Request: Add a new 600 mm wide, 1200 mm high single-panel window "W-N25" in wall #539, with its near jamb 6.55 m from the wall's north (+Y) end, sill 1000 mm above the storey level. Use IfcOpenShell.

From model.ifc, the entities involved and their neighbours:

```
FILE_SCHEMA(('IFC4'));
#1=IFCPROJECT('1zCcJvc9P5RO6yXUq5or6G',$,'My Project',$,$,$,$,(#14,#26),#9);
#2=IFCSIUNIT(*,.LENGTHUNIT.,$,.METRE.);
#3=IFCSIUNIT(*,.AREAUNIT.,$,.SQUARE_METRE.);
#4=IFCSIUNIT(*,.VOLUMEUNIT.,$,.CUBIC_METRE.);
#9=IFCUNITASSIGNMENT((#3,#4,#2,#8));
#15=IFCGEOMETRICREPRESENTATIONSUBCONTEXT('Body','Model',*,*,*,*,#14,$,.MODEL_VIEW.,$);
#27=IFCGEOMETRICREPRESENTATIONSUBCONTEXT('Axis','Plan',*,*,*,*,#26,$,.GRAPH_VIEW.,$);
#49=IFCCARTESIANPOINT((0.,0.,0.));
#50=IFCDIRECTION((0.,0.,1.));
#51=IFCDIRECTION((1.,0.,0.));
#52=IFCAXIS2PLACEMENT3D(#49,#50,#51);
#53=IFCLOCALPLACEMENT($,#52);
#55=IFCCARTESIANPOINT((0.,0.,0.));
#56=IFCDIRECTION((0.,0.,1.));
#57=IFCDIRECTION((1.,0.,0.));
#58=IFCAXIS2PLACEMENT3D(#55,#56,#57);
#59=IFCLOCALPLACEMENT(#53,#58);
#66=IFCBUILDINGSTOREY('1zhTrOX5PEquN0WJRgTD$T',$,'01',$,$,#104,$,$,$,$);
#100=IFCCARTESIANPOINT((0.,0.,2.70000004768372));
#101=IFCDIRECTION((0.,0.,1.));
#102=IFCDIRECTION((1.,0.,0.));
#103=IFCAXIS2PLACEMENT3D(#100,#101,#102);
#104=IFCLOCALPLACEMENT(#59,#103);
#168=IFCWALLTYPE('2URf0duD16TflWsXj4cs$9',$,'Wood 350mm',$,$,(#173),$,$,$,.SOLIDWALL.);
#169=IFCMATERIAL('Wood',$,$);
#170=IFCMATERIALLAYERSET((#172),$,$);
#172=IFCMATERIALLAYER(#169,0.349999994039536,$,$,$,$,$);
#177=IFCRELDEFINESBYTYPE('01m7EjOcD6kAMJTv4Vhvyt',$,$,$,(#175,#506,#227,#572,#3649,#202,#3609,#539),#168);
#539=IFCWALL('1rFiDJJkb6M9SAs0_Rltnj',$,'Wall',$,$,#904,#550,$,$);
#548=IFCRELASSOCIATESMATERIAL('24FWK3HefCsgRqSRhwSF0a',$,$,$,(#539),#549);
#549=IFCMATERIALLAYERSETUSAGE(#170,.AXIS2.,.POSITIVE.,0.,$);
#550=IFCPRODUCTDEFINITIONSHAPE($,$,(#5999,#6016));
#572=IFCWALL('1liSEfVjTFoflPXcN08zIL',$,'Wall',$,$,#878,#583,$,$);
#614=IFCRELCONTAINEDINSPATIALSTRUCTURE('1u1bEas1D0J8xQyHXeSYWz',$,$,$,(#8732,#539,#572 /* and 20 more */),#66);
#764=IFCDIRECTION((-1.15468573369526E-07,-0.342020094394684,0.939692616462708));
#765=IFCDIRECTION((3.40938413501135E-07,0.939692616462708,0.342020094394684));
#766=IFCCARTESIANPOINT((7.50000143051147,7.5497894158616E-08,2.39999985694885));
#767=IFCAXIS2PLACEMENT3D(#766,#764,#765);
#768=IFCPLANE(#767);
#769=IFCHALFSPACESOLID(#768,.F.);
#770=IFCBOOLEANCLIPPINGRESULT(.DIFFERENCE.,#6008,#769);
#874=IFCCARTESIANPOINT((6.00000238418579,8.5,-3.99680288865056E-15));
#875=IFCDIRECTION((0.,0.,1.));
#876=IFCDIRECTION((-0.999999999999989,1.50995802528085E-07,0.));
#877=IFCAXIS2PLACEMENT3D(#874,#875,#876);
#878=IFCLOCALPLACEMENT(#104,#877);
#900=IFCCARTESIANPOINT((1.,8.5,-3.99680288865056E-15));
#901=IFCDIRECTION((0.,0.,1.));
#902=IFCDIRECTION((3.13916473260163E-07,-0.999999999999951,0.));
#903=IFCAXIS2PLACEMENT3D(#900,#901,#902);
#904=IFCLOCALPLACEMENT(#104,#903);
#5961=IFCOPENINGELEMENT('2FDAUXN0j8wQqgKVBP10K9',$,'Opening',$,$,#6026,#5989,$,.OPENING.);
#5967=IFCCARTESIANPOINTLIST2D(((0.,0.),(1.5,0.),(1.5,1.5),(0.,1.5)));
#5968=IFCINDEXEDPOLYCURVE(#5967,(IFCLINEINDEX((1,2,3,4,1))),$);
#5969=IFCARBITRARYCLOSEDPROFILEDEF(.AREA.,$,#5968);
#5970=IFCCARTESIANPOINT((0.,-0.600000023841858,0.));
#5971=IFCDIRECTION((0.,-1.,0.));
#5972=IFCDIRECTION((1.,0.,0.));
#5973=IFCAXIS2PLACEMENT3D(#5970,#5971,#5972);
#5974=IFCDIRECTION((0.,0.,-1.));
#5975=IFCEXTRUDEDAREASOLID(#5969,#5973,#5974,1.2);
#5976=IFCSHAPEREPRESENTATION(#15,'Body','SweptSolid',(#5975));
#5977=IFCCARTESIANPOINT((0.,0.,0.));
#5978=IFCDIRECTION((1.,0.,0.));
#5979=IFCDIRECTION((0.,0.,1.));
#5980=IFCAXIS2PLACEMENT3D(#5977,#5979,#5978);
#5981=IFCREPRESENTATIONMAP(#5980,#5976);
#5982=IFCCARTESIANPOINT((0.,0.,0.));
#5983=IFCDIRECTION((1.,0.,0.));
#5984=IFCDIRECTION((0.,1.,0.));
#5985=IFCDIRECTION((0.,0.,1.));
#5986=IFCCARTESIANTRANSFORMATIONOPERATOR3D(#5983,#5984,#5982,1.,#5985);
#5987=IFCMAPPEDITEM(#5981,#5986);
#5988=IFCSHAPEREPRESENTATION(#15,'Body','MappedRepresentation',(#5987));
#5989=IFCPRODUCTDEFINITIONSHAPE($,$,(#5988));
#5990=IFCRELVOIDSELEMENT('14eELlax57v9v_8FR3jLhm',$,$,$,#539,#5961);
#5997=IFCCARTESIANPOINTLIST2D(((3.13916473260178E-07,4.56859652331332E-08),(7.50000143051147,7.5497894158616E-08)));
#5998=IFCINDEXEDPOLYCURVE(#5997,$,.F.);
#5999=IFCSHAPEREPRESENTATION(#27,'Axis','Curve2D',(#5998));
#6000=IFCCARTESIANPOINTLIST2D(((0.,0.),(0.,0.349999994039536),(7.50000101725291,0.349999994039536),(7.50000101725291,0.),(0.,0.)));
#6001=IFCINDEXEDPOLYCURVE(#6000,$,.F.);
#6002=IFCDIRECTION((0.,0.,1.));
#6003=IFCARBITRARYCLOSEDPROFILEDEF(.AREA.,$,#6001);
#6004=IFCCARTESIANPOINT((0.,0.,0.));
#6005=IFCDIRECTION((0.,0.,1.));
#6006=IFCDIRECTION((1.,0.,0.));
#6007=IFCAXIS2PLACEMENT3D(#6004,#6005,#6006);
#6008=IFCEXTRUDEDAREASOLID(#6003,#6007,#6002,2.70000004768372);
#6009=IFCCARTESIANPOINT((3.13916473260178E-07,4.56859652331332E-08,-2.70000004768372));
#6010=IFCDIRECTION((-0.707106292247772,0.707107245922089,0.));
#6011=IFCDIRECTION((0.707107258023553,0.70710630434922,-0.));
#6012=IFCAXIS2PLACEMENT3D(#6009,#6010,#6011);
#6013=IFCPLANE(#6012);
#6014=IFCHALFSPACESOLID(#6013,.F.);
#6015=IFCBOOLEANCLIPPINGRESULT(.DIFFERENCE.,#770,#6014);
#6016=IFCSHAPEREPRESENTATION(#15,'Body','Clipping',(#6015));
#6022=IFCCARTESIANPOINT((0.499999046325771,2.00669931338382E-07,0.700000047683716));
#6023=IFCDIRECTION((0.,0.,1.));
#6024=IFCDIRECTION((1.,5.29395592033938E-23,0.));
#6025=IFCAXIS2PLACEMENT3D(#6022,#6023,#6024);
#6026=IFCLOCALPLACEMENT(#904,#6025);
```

```python
import numpy as np
import ifcopenshell
import ifcopenshell.api.feature
import ifcopenshell.api.geometry
import ifcopenshell.api.root
import ifcopenshell.api.spatial
import ifcopenshell.geom
import ifcopenshell.util.element
import ifcopenshell.util.placement
import ifcopenshell.util.representation
import ifcopenshell.util.shape
import ifcopenshell.util.unit

model = ifcopenshell.open("model.ifc")
unit_scale = ifcopenshell.util.unit.calculate_unit_scale(model)
settings = ifcopenshell.geom.settings()


def volume(element):
    """Net volume in cubic metres, openings subtracted."""
    shape = ifcopenshell.geom.create_shape(settings, element)
    return ifcopenshell.util.shape.get_volume(shape.geometry)


wall = model.by_id(539)
storey = ifcopenshell.util.element.get_container(wall, ifc_class="IfcBuildingStorey")
context = ifcopenshell.util.representation.get_context(model, "Model", "Body", "MODEL_VIEW")
before = volume(wall)

width, height, from_end, sill = 0.6, 1.2, 6.55, 1  # metres

# The wall runs along its own X axis, and the end named is its -X end.
wall_shape = ifcopenshell.geom.create_shape(settings, wall)
x, y, z = ifcopenshell.util.shape.get_vertices(wall_shape.geometry).T
start = x.min() + from_end
face, thickness = float(y.min()), float(y.max() - y.min())
wall_matrix = ifcopenshell.util.placement.get_local_placement(wall.ObjectPlacement)
level = ifcopenshell.util.placement.get_local_placement(storey.ObjectPlacement)[2, 3]


def in_wall(x, y):
    """Placement at x, y metres in the wall's axes, at sill height."""
    matrix = wall_matrix.copy()
    matrix[:, 3] = wall_matrix @ np.array([x / unit_scale, y / unit_scale, 0.0, 1.0])
    matrix[2, 3] = level + sill / unit_scale
    return matrix


# Opening: a box that overshoots both wall faces by 50 mm.
opening = ifcopenshell.api.root.create_entity(model, ifc_class="IfcOpeningElement", predefined_type="OPENING")
box = ifcopenshell.api.geometry.add_wall_representation(
    model, context=context, length=width, height=height, thickness=thickness + 0.1
)
ifcopenshell.api.geometry.assign_representation(model, product=opening, representation=box)
ifcopenshell.api.geometry.edit_object_placement(model, product=opening, matrix=in_wall(start, face - 0.05), is_si=False)
ifcopenshell.api.feature.add_feature(model, feature=opening, element=wall)

window = ifcopenshell.api.root.create_entity(model, ifc_class="IfcWindow", name="W-N25", predefined_type="WINDOW")
window.OverallWidth, window.OverallHeight = width / unit_scale, height / unit_scale
window.PartitioningType = "SINGLE_PANEL"
body = ifcopenshell.api.geometry.add_window_representation(
    model,
    context=context,
    overall_width=window.OverallWidth,
    overall_height=window.OverallHeight,
    partition_type="SINGLE_PANEL",
)
ifcopenshell.api.geometry.assign_representation(model, product=window, representation=body)
ifcopenshell.api.spatial.assign_container(model, products=[window], relating_structure=storey)
ifcopenshell.api.feature.add_filling(model, opening=opening, element=window)

# Centre the window in the wall's thickness.
ifcopenshell.api.geometry.edit_object_placement(model, product=window, matrix=in_wall(start, face), is_si=False)
window_shape = ifcopenshell.geom.create_shape(settings, window)
depth = ifcopenshell.util.shape.get_vertices(window_shape.geometry)[:, 1]
offset = face + thickness / 2 - (depth.min() + depth.max()) / 2
ifcopenshell.api.geometry.edit_object_placement(model, product=window, matrix=in_wall(start, offset), is_si=False)

after = volume(wall)

print(f"wall volume {before:.3f} -> {after:.3f} m3")

model.write("model_edited.ifc")
```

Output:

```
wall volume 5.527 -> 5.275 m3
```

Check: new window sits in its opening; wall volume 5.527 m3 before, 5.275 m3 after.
